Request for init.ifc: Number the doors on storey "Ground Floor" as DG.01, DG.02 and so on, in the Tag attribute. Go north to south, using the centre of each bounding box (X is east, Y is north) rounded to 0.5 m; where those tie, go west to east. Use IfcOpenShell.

First a look at what the model holds.

```python
import ifcopenshell
import ifcopenshell.util.element
import ifcopenshell.util.placement

model = ifcopenshell.open("init.ifc")
print(model.schema)
storey = next(s for s in model.by_type("IfcBuildingStorey") if s.Name == "Ground Floor")
doors = [e for e in ifcopenshell.util.element.get_decomposition(storey) if e.is_a("IfcDoor")]
for e in sorted(doors, key=lambda e: e.id()):
    origin = ifcopenshell.util.placement.get_local_placement(e.ObjectPlacement)[:3, 3]
    print(e.id(), e.Tag, e.Name, origin.round(2) + 0.0, sep=" | ")
```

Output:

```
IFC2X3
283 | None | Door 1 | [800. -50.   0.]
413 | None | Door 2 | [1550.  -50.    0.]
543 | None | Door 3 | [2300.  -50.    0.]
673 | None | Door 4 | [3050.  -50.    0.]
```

```python
import ifcopenshell
import ifcopenshell.geom
import ifcopenshell.util.element
import ifcopenshell.util.shape

model = ifcopenshell.open("init.ifc")
settings = ifcopenshell.geom.settings()
settings.set("use-world-coords", True)


def centre(element):
    shape = ifcopenshell.geom.create_shape(settings, element)
    return ifcopenshell.util.shape.get_bbox_centroid(shape.geometry)


storey = next(s for s in model.by_type("IfcBuildingStorey") if s.Name == "Ground Floor")
doors = [e for e in ifcopenshell.util.element.get_decomposition(storey) if e.is_a("IfcDoor")]

# Insertion points can sit at a corner or the storey origin, so sort by the geometry (in metres).
centres = {e: centre(e) for e in doors}
doors.sort(key=lambda e: (-round(centres[e][1] / 0.5), centres[e][0]))

for i, e in enumerate(doors, start=1):
    number = f"DG.{i:02d}"
    e.Tag = number
    print(e.id(), number)

model.write("init-out.ifc")
```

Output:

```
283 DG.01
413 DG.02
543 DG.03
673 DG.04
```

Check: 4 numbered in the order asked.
